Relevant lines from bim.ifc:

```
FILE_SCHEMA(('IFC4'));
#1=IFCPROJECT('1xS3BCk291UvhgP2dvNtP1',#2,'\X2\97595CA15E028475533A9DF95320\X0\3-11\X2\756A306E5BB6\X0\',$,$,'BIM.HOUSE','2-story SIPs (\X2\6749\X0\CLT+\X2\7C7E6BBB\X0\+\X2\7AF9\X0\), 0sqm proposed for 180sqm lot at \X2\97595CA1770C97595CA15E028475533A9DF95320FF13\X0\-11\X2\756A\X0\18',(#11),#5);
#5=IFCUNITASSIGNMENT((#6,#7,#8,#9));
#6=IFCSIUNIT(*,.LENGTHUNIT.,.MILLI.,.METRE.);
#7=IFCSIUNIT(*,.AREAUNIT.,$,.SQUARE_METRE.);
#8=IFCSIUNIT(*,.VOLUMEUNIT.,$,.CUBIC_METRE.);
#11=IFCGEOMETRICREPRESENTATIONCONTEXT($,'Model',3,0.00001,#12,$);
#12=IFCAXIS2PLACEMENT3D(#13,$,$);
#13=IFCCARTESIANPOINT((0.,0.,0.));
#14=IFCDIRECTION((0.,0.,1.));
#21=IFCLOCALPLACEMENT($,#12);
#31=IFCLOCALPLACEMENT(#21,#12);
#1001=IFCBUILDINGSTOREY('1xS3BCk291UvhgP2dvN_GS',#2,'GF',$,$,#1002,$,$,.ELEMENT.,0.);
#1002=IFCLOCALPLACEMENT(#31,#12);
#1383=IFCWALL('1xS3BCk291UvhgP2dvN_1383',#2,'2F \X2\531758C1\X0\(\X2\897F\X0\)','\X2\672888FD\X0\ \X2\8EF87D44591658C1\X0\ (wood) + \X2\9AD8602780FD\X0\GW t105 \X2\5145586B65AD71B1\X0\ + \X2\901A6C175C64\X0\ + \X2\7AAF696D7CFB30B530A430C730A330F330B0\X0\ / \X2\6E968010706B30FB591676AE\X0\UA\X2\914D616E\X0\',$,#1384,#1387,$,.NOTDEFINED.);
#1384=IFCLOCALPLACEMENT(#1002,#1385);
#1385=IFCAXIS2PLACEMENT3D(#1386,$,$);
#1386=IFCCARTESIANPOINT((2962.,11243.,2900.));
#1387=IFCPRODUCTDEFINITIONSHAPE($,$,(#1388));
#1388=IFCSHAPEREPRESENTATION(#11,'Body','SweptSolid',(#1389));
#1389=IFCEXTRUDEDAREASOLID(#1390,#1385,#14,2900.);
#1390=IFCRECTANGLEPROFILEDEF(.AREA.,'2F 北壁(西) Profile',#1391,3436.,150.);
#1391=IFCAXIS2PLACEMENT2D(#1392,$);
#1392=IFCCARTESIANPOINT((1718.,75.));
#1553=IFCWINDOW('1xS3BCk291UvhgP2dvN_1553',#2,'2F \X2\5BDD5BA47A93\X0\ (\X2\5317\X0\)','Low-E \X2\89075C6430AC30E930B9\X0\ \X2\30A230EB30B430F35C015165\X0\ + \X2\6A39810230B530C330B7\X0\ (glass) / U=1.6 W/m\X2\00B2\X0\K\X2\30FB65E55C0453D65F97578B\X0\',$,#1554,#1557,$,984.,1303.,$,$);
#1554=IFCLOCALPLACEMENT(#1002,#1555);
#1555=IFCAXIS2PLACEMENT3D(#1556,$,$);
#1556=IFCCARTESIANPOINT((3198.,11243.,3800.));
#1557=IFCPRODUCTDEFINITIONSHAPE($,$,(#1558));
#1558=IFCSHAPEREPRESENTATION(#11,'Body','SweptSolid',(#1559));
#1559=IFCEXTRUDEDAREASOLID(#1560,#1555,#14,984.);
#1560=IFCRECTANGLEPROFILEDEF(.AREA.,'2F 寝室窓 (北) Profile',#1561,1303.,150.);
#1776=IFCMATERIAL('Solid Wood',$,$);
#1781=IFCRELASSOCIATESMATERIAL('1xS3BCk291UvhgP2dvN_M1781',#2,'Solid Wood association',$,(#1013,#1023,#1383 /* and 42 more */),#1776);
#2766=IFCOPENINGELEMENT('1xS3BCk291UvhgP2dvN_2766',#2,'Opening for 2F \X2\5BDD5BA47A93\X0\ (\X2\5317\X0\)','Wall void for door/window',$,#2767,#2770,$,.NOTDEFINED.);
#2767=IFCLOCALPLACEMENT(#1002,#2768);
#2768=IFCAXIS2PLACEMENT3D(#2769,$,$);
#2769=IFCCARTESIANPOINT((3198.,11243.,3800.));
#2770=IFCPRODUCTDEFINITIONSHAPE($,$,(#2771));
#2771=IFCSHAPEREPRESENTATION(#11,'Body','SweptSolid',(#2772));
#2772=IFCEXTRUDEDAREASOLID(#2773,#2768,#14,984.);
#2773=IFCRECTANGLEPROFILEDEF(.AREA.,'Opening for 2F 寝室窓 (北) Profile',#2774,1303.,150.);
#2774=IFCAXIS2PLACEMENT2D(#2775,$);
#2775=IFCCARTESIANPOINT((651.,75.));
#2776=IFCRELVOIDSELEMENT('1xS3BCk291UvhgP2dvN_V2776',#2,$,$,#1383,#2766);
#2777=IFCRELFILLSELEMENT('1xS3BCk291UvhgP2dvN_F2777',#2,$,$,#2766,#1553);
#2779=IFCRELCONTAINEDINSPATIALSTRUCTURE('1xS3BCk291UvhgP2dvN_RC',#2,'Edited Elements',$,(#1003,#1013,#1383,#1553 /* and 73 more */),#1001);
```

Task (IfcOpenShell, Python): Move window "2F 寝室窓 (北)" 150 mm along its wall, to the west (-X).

```python
import ifcopenshell
import ifcopenshell.api.geometry
import ifcopenshell.util.placement
import ifcopenshell.util.unit

model = ifcopenshell.open("bim.ifc")
unit_scale = ifcopenshell.util.unit.calculate_unit_scale(model)

window = model.by_guid("1xS3BCk291UvhgP2dvN_1553")
opening = window.FillsVoids[0].RelatingOpeningElement
wall = opening.VoidsElements[0].RelatingBuildingElement

wall_matrix = ifcopenshell.util.placement.get_local_placement(wall.ObjectPlacement)
shift = wall_matrix[:3, 0] * -0.15 / unit_scale
before = ifcopenshell.util.placement.get_local_placement(window.ObjectPlacement)[:3, 3].copy()

# The window is not placed relative to its opening, so move both.
for product in (opening, window):
    matrix = ifcopenshell.util.placement.get_local_placement(product.ObjectPlacement)
    matrix[:3, 3] += shift
    ifcopenshell.api.geometry.edit_object_placement(model, product=product, matrix=matrix, is_si=False)

after = ifcopenshell.util.placement.get_local_placement(window.ObjectPlacement)[:3, 3]
print("window moved by", (after - before).round(3) + 0.0)

model.write("bim_rev.ifc")
```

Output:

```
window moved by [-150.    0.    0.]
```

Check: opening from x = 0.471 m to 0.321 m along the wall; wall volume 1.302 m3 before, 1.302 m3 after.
